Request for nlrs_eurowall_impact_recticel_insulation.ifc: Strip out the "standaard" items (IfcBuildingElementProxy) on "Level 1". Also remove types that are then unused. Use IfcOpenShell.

First a look at what the model holds.

```python
import ifcopenshell
import ifcopenshell.util.element

model = ifcopenshell.open("nlrs_eurowall_impact_recticel_insulation.ifc")
print(model.schema)
storey = next(s for s in model.by_type("IfcBuildingStorey") if s.Name == "Level 1")
proxies = [e for e in ifcopenshell.util.element.get_decomposition(storey) if e.is_a("IfcBuildingElementProxy")]
seen = {}
for e in proxies:
    element_type = ifcopenshell.util.element.get_type(e)
    name = element_type.Name if element_type not in (None, e) else None
    seen[name] = seen.get(name, 0) + 1
for name, count in sorted(seen.items(), key=str):
    print(count, "x", name)
```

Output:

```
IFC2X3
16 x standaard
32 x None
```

```python
import ifcopenshell
import ifcopenshell.api.root
import ifcopenshell.util.element

model = ifcopenshell.open("nlrs_eurowall_impact_recticel_insulation.ifc")

storey = next(s for s in model.by_type("IfcBuildingStorey") if s.Name == "Level 1")
proxies = [e for e in ifcopenshell.util.element.get_decomposition(storey) if e.is_a("IfcBuildingElementProxy")]
targets = [e for e in proxies if (t := ifcopenshell.util.element.get_type(e)) not in (None, e) and t.Name == "standaard"]
types = {ifcopenshell.util.element.get_type(e) for e in targets} - {None, *targets}

for e in targets:
    ifcopenshell.api.root.remove_product(model, product=e)
print(len(targets), "removed")

unused = [t for t in types if not ifcopenshell.util.element.get_types(t)]
for t in unused:
    ifcopenshell.api.root.remove_product(model, product=t)
print(len(unused), "unused types removed")

model.write("nlrs_eurowall_impact_recticel_insulation_edited.ifc")
```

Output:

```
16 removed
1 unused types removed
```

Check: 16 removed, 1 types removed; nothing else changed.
